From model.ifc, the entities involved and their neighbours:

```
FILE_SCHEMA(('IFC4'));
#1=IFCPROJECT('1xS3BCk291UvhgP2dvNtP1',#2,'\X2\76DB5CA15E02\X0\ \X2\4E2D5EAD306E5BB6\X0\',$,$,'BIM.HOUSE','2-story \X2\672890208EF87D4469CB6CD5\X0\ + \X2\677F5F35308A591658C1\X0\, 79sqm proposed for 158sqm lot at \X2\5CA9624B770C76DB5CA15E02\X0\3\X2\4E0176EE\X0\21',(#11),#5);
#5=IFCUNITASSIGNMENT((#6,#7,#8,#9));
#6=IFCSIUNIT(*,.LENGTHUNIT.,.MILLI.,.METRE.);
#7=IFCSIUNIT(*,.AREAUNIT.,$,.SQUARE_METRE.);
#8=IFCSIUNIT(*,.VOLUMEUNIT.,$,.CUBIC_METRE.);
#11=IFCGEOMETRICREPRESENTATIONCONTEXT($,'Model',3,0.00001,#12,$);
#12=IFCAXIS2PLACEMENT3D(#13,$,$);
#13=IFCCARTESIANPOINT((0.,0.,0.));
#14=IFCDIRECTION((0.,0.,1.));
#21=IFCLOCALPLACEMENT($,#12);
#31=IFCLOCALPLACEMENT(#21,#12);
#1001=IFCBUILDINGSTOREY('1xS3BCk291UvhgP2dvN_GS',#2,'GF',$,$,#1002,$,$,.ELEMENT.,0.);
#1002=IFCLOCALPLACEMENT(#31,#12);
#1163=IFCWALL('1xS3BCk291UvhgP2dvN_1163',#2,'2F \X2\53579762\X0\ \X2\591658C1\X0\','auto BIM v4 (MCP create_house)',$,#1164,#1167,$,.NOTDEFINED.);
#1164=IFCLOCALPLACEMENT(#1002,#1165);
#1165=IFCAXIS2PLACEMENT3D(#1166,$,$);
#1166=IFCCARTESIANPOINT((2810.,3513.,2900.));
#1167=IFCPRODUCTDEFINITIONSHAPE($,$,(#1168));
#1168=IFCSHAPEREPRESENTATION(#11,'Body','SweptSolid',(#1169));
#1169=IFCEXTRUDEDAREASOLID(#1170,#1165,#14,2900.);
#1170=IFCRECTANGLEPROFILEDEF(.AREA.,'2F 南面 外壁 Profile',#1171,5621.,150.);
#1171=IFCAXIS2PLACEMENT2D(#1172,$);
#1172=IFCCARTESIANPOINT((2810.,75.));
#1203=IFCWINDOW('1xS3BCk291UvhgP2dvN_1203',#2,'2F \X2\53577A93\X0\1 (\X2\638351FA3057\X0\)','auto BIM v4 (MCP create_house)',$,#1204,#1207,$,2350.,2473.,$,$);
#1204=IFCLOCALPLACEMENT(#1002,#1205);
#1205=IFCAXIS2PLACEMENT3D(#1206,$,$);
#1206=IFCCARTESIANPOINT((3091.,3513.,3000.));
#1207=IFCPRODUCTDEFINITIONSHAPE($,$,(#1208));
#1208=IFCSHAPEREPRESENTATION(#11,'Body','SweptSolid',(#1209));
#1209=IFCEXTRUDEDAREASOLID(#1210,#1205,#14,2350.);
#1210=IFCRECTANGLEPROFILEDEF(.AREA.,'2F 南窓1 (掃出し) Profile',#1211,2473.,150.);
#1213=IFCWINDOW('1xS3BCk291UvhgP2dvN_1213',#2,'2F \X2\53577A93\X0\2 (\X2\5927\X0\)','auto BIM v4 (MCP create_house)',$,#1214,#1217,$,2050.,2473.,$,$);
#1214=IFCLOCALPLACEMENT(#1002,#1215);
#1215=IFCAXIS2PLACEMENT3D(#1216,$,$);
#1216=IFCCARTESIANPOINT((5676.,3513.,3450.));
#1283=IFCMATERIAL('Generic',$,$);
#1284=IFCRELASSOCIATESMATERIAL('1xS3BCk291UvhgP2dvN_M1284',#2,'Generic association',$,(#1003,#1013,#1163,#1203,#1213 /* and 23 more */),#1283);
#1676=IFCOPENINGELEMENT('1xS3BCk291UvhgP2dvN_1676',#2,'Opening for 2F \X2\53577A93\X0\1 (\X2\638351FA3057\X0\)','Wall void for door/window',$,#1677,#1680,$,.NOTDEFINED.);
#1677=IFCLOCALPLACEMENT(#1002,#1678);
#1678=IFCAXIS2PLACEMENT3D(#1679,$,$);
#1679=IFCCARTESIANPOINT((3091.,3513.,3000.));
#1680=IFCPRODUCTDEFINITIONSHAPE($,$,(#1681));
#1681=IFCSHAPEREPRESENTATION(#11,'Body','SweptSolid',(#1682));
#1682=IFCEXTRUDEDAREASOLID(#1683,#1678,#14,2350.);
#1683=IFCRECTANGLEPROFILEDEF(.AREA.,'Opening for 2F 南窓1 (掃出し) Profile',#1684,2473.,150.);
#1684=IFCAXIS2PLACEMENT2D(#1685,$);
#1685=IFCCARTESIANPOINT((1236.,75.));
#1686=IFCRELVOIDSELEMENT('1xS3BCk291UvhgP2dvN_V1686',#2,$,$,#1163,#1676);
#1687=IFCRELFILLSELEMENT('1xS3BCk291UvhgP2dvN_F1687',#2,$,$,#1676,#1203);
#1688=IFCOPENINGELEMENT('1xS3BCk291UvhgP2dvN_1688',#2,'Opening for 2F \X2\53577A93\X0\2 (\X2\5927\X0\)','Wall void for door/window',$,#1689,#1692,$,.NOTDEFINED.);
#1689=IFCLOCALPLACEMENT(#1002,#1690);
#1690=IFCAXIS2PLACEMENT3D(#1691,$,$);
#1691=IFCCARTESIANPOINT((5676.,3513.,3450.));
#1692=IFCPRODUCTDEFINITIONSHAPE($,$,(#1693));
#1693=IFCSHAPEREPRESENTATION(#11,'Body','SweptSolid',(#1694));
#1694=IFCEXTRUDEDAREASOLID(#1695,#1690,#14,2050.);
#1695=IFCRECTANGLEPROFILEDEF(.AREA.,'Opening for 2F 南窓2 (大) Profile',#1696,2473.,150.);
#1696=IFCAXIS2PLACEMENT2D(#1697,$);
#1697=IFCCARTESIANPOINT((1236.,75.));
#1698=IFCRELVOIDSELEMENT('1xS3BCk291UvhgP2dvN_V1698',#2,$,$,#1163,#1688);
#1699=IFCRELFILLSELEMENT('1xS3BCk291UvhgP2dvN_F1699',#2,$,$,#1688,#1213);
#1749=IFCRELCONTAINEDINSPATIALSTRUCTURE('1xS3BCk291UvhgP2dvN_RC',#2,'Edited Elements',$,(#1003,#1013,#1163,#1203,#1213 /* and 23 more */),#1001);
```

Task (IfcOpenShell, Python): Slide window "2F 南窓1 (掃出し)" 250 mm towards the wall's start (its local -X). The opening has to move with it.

```python
import ifcopenshell
import ifcopenshell.api.geometry
import ifcopenshell.util.placement
import ifcopenshell.util.unit

model = ifcopenshell.open("model.ifc")
unit_scale = ifcopenshell.util.unit.calculate_unit_scale(model)

window = model.by_guid("1xS3BCk291UvhgP2dvN_1203")
opening = window.FillsVoids[0].RelatingOpeningElement
wall = opening.VoidsElements[0].RelatingBuildingElement

wall_matrix = ifcopenshell.util.placement.get_local_placement(wall.ObjectPlacement)
shift = wall_matrix[:3, 0] * -0.25 / unit_scale
before = ifcopenshell.util.placement.get_local_placement(window.ObjectPlacement)[:3, 3].copy()

# The window is not placed relative to its opening, so move both.
for product in (opening, window):
    matrix = ifcopenshell.util.placement.get_local_placement(product.ObjectPlacement)
    matrix[:3, 3] += shift
    ifcopenshell.api.geometry.edit_object_placement(model, product=product, matrix=matrix, is_si=False)

after = ifcopenshell.util.placement.get_local_placement(window.ObjectPlacement)[:3, 3]
print("window moved by", (after - before).round(3) + 0.0)

model.write("model_rev.ifc")
```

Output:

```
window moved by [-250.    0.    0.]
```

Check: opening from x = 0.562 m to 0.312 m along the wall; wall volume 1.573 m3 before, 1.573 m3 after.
